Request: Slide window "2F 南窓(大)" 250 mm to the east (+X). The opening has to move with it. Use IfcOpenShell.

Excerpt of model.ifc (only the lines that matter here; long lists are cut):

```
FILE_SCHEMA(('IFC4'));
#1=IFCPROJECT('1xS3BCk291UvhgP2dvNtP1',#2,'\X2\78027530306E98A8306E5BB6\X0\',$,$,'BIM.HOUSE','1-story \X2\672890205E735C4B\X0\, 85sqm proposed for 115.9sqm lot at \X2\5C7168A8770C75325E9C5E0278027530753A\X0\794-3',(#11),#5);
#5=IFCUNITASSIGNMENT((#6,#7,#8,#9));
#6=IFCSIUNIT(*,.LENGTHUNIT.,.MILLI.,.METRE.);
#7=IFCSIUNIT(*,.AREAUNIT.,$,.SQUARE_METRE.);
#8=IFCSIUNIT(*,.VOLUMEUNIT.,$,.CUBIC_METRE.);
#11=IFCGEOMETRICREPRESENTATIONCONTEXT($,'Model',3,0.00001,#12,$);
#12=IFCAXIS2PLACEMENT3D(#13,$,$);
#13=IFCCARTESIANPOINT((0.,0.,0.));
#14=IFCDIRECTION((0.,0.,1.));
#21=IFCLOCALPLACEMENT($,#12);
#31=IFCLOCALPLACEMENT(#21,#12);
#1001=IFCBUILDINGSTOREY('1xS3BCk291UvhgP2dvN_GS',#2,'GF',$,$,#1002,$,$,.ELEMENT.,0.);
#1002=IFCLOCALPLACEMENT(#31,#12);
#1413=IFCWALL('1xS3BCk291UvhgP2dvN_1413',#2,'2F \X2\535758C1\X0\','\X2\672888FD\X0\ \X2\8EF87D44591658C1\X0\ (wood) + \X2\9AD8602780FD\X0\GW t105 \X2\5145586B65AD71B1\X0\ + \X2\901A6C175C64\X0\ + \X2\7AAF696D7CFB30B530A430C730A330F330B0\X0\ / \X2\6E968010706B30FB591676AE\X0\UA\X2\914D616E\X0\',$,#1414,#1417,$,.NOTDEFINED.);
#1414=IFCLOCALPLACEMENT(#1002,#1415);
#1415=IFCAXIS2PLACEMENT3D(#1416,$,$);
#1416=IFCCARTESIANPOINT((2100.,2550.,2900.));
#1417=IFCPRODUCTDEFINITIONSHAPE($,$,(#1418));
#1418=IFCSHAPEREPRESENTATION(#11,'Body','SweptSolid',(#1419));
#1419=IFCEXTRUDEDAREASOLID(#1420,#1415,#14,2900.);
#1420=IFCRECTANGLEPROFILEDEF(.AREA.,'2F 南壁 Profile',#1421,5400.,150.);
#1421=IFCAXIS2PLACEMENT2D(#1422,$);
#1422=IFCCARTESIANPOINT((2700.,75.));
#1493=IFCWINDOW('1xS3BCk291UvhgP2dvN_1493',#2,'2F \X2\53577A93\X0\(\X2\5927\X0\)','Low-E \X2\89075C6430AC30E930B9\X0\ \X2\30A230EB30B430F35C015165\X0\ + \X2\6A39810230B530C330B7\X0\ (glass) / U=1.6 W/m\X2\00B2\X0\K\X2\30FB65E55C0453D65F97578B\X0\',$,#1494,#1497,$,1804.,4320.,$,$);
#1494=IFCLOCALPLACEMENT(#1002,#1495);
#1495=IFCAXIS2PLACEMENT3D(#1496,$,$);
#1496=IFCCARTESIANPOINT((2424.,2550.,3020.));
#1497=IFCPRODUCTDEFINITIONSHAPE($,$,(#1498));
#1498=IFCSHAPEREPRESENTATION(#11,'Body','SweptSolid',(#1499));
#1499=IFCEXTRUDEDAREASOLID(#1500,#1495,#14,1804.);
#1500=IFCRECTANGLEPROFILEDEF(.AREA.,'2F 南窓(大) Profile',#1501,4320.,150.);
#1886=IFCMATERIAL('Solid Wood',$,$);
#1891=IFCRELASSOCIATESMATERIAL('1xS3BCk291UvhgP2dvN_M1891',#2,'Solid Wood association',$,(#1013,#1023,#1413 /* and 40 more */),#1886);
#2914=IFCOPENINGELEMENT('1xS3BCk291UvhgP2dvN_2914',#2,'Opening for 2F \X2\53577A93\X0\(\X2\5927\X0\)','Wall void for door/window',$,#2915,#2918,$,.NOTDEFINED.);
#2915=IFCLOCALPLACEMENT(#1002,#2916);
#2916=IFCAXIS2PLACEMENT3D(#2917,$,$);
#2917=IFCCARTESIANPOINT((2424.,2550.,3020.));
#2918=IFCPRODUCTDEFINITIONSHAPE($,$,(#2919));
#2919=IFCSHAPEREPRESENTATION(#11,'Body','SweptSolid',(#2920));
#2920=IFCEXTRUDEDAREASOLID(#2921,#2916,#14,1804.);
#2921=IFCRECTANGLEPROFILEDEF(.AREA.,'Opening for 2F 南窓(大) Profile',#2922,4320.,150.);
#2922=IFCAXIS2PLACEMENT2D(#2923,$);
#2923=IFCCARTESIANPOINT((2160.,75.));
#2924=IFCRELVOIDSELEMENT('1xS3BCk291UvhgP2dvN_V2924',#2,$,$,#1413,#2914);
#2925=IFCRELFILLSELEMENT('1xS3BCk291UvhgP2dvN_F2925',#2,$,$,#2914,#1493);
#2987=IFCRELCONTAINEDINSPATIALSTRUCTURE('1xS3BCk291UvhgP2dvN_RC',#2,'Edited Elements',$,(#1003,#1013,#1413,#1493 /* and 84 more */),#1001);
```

```python
import ifcopenshell
import ifcopenshell.api.geometry
import ifcopenshell.util.placement
import ifcopenshell.util.unit

model = ifcopenshell.open("model.ifc")
unit_scale = ifcopenshell.util.unit.calculate_unit_scale(model)

window = model.by_guid("1xS3BCk291UvhgP2dvN_1493")
opening = window.FillsVoids[0].RelatingOpeningElement
wall = opening.VoidsElements[0].RelatingBuildingElement

wall_matrix = ifcopenshell.util.placement.get_local_placement(wall.ObjectPlacement)
shift = wall_matrix[:3, 0] * 0.25 / unit_scale
before = ifcopenshell.util.placement.get_local_placement(window.ObjectPlacement)[:3, 3].copy()

# The window is not placed relative to its opening, so move both.
for product in (opening, window):
    matrix = ifcopenshell.util.placement.get_local_placement(product.ObjectPlacement)
    matrix[:3, 3] += shift
    ifcopenshell.api.geometry.edit_object_placement(model, product=product, matrix=matrix, is_si=False)

after = ifcopenshell.util.placement.get_local_placement(window.ObjectPlacement)[:3, 3]
print("window moved by", (after - before).round(3) + 0.0)

model.write("model_rev.ifc")
```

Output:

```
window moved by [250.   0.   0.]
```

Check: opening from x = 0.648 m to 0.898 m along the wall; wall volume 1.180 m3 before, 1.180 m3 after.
